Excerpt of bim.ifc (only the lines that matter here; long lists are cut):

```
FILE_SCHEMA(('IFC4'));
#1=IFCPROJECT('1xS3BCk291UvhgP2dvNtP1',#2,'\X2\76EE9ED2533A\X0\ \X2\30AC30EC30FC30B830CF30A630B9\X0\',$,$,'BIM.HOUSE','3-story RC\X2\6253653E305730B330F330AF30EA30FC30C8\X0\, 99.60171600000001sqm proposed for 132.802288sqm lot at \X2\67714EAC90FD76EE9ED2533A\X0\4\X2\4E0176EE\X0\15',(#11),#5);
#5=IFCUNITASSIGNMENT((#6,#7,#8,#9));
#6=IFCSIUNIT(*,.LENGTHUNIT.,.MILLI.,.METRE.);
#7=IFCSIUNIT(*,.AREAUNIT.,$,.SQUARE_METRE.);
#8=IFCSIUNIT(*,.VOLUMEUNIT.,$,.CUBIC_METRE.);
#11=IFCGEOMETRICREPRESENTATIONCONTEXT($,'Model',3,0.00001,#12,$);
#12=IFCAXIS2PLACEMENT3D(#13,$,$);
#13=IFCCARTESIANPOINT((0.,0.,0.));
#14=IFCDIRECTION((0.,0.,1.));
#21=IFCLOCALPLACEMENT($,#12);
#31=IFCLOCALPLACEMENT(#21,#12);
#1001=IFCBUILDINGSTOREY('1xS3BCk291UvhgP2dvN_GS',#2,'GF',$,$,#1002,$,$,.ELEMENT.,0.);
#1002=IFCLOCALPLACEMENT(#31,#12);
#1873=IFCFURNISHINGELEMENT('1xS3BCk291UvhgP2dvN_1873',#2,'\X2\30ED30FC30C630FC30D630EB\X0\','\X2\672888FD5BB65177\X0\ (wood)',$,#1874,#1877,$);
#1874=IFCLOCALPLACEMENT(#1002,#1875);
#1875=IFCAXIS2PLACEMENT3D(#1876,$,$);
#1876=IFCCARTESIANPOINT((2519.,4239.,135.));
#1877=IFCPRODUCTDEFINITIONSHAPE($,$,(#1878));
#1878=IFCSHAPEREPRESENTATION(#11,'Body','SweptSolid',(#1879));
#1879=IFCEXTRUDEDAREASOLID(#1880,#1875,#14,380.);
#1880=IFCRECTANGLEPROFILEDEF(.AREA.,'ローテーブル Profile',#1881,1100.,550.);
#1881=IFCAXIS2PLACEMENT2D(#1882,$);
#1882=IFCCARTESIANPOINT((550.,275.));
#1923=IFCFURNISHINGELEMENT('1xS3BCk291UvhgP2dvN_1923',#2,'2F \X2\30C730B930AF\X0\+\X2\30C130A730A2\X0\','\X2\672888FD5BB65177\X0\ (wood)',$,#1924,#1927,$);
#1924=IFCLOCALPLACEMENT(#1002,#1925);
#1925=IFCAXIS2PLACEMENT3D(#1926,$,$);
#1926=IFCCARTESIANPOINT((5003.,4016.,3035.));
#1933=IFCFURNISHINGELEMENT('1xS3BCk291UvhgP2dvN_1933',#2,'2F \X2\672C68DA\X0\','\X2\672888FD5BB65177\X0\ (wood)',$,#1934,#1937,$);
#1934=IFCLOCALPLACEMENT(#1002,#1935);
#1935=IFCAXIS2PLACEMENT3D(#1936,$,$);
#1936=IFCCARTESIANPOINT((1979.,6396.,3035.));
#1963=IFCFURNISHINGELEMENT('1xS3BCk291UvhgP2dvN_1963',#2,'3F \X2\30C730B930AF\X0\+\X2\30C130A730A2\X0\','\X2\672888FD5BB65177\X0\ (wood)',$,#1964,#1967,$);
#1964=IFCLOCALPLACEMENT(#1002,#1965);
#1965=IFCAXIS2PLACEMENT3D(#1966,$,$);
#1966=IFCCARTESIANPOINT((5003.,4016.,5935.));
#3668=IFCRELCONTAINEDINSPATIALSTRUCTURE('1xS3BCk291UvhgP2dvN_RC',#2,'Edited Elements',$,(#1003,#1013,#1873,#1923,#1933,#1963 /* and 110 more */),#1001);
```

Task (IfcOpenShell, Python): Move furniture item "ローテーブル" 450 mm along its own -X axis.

```python
import ifcopenshell
import ifcopenshell.api.geometry
import ifcopenshell.util.placement
import ifcopenshell.util.unit

model = ifcopenshell.open("bim.ifc")
unit_scale = ifcopenshell.util.unit.calculate_unit_scale(model)

item = model.by_id(1873)
matrix = ifcopenshell.util.placement.get_local_placement(item.ObjectPlacement)
matrix[:3, 3] -= matrix[:3, 0] * 0.45 / unit_scale
ifcopenshell.api.geometry.edit_object_placement(model, product=item, matrix=matrix, is_si=False)

print(ifcopenshell.util.placement.get_local_placement(item.ObjectPlacement).round(3) + 0.0)

model.write("bim_rev.ifc")
```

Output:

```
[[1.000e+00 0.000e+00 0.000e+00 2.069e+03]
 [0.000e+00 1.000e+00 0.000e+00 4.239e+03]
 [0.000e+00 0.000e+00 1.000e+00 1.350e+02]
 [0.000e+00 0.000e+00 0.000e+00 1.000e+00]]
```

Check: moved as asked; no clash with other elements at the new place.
